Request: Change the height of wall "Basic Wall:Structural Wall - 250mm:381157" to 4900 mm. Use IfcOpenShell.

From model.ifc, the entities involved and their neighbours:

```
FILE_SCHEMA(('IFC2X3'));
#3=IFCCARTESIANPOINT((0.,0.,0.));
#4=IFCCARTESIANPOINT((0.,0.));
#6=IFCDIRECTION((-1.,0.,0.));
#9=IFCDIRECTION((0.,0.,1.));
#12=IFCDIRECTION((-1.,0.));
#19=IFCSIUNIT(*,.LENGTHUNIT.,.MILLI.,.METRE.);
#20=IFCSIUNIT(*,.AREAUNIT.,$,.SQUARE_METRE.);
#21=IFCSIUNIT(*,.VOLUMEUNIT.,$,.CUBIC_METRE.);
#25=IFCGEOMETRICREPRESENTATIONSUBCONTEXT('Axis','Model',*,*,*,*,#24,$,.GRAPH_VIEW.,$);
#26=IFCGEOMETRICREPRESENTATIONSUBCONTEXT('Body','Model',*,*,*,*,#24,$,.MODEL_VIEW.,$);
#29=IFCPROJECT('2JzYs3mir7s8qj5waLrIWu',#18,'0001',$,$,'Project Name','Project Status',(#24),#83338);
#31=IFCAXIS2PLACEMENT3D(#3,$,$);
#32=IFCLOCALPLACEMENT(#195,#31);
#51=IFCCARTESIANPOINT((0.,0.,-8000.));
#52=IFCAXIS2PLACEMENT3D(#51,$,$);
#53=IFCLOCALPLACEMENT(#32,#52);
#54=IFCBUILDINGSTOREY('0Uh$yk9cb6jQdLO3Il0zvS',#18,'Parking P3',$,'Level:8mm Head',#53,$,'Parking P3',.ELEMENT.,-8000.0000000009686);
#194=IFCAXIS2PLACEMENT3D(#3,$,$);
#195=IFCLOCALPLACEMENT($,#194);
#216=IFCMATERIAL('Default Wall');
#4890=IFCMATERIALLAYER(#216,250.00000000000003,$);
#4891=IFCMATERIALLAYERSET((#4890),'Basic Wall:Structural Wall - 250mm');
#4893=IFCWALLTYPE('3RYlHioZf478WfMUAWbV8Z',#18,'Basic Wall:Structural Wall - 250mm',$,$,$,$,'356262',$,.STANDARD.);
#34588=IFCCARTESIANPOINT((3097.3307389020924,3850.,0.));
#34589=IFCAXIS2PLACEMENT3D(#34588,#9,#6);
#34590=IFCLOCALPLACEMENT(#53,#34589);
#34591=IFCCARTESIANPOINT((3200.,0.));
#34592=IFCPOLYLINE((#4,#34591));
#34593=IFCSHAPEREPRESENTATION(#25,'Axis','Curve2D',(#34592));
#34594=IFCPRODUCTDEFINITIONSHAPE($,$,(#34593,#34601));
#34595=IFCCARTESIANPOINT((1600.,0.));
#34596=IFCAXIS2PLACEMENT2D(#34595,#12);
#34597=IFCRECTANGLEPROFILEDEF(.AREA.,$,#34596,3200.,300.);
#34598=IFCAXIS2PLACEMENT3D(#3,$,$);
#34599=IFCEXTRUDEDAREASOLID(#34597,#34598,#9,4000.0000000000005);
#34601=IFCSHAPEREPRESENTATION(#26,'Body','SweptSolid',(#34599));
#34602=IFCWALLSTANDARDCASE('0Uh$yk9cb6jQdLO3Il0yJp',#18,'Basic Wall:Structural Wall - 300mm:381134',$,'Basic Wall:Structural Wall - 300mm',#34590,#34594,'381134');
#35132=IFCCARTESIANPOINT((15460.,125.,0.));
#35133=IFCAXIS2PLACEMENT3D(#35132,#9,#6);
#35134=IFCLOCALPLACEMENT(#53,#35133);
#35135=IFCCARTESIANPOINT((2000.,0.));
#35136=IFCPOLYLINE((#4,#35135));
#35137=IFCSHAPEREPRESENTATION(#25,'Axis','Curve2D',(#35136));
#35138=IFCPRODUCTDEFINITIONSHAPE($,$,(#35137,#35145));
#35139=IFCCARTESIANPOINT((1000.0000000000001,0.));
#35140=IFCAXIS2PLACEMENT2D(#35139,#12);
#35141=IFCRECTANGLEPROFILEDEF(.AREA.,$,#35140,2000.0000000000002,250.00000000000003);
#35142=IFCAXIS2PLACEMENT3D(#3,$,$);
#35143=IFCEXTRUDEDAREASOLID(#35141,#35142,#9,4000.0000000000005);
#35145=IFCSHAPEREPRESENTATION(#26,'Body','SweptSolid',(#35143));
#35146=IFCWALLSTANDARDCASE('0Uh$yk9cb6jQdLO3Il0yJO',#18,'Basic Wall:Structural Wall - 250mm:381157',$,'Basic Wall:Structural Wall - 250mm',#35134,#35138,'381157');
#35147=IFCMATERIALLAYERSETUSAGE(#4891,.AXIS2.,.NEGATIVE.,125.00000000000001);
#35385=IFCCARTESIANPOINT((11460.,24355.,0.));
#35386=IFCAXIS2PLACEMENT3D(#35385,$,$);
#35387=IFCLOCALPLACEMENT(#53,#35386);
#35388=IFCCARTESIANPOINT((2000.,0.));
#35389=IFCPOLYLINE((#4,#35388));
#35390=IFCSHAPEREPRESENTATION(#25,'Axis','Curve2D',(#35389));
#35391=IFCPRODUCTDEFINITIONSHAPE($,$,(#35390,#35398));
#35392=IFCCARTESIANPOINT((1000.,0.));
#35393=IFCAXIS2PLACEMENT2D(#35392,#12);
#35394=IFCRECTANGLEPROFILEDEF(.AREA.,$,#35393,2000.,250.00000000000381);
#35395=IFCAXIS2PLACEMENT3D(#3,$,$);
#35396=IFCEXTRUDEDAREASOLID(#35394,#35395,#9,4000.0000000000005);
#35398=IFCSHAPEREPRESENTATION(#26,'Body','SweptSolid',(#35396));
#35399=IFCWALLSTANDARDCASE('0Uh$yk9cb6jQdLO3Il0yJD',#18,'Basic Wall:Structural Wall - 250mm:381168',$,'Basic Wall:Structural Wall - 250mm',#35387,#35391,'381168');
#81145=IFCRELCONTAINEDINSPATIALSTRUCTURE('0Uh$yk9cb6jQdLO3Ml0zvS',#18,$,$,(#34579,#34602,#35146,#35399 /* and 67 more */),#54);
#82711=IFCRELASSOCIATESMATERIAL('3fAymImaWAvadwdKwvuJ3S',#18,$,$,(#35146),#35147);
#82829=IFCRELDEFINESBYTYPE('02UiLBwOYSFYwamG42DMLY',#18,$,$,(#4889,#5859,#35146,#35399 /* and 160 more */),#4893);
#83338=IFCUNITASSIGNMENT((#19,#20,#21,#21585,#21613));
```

```python
import ifcopenshell
import ifcopenshell.geom
import ifcopenshell.util.representation
import ifcopenshell.util.shape

model = ifcopenshell.open("model.ifc")
settings = ifcopenshell.geom.settings()


def volume(element):
    """Net volume in cubic metres, openings subtracted."""
    shape = ifcopenshell.geom.create_shape(settings, element)
    return ifcopenshell.util.shape.get_volume(shape.geometry)


wall = model.by_guid("0Uh$yk9cb6jQdLO3Il0yJO")
before = volume(wall)

body = ifcopenshell.util.representation.get_representation(wall, "Model", "Body")
solid = body.Items[0]
old_height = solid.Depth
solid.Depth = 4900.0
after = volume(wall)

print(f"height {old_height:g} -> {solid.Depth:g}, volume {before:.3f} -> {after:.3f} m3")

model.write("model_edited.ifc")
```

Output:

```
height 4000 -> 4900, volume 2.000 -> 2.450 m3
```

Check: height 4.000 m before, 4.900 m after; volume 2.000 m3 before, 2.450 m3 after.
